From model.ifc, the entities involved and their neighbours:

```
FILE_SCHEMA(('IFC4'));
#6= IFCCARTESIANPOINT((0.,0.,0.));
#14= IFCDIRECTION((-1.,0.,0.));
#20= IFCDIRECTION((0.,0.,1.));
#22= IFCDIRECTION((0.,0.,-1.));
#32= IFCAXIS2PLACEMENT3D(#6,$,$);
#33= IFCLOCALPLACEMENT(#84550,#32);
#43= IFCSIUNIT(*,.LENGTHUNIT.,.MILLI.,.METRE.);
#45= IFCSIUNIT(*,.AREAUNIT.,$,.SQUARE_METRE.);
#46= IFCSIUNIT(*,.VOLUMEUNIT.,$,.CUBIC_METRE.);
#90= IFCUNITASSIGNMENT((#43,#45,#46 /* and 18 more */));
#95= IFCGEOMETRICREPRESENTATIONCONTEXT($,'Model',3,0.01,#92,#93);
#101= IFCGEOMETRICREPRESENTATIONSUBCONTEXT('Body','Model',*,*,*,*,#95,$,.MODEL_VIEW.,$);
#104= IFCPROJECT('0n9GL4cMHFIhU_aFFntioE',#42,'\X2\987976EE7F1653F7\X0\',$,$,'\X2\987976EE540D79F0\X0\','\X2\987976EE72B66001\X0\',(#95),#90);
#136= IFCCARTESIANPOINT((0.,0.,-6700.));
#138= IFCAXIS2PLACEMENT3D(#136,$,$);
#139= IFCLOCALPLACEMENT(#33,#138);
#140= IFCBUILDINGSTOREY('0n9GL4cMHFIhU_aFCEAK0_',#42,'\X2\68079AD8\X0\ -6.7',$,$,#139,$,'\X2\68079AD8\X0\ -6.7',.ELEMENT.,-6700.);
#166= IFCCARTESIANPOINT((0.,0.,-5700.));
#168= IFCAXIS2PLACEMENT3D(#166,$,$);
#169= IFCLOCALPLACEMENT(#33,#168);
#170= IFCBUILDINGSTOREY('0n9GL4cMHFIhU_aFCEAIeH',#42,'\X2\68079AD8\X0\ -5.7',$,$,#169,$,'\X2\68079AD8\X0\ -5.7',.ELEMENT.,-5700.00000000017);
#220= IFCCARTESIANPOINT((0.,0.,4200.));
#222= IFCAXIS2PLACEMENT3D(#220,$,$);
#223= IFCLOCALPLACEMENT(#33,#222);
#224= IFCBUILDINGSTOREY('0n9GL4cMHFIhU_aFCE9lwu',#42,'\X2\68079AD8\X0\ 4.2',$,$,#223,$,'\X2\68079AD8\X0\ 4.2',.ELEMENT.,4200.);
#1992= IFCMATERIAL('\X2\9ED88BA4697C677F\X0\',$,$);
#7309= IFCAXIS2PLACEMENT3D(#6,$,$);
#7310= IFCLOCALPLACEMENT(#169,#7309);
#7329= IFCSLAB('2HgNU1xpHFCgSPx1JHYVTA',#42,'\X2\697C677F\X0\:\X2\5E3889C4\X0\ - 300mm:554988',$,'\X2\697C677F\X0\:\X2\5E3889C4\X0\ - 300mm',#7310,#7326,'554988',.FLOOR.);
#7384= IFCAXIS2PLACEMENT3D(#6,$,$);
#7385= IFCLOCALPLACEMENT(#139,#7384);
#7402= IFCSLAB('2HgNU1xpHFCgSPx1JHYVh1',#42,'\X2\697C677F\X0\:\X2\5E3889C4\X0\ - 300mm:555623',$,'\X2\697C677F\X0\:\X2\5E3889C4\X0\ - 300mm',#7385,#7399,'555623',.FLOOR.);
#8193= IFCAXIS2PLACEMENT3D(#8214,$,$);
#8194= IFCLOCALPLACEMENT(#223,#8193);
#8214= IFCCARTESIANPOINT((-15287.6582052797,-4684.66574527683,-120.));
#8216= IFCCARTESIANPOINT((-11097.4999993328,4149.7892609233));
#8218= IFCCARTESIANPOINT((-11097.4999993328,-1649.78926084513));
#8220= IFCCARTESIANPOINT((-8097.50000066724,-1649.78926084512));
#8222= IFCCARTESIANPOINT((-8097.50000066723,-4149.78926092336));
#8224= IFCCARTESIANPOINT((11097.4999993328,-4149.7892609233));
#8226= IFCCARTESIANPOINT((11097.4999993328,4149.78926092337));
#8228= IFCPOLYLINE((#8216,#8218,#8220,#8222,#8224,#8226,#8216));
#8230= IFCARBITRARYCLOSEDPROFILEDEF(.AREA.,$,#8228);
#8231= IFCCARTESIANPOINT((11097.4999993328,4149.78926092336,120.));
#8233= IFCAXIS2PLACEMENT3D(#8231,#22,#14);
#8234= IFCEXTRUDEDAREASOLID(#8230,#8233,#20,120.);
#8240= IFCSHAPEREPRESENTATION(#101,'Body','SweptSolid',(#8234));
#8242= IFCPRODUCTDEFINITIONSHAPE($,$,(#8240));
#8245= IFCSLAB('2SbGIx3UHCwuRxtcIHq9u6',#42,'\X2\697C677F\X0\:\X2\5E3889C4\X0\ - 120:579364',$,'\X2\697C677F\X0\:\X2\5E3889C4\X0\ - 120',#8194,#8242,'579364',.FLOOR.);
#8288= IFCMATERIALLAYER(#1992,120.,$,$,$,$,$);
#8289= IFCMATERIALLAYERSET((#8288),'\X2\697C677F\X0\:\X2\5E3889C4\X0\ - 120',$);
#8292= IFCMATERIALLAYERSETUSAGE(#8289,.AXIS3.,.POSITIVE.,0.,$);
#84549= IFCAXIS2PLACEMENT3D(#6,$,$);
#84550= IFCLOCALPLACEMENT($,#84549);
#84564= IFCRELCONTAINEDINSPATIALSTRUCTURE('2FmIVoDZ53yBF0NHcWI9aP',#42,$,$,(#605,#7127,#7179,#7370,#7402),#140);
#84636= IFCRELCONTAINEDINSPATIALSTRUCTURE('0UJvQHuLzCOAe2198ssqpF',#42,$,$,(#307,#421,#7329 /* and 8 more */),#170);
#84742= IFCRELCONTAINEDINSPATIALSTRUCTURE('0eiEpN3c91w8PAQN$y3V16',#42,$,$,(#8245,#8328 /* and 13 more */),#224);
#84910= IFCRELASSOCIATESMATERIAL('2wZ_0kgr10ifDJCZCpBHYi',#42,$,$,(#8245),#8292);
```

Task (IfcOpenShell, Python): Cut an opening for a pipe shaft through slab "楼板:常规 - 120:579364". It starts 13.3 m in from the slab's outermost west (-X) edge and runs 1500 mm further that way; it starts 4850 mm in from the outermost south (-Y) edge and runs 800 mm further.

```python
import numpy as np
import ifcopenshell
import ifcopenshell.api.feature
import ifcopenshell.api.geometry
import ifcopenshell.api.root
import ifcopenshell.geom
import ifcopenshell.util.placement
import ifcopenshell.util.representation
import ifcopenshell.util.shape
import ifcopenshell.util.unit

model = ifcopenshell.open("model.ifc")
unit_scale = ifcopenshell.util.unit.calculate_unit_scale(model)
settings = ifcopenshell.geom.settings()


def volume(element):
    """Net volume in cubic metres, openings subtracted."""
    shape = ifcopenshell.geom.create_shape(settings, element)
    return ifcopenshell.util.shape.get_volume(shape.geometry)


slab = model.by_guid("2SbGIx3UHCwuRxtcIHq9u6")
before = volume(slab)

# Extent in the slab's own axes, in metres. The edges named are its -X and -Y sides.
slab_shape = ifcopenshell.geom.create_shape(settings, slab)
vertices = ifcopenshell.util.shape.get_vertices(slab_shape.geometry)
x_min, y_min, bottom = vertices.min(axis=0)
top = vertices[:, 2].max()

opening = ifcopenshell.api.root.create_entity(model, ifc_class="IfcOpeningElement", name="Pipe shaft opening", predefined_type="OPENING")
context = ifcopenshell.util.representation.get_context(model, "Model", "Body", "MODEL_VIEW")
width, depth = 1.5, 0.8
outline = [(0.0, 0.0), (width, 0.0), (width, depth), (0.0, depth), (0.0, 0.0)]
# Overshoot both faces by 50 mm so the cut is clean.
shape = ifcopenshell.api.geometry.add_slab_representation(
    model, context=context, depth=top - bottom + 0.1, polyline=outline
)
ifcopenshell.api.geometry.assign_representation(model, product=opening, representation=shape)

matrix = ifcopenshell.util.placement.get_local_placement(slab.ObjectPlacement)
matrix[:, 3] = matrix @ np.append(np.array([x_min + 13.3, y_min + 4.85, bottom - 0.05]) / unit_scale, 1.0)
ifcopenshell.api.geometry.edit_object_placement(model, product=opening, matrix=matrix, is_si=False)
ifcopenshell.api.feature.add_feature(model, feature=opening, element=slab)

after = volume(slab)

print(f"slab volume {before:.3f} -> {after:.3f} m3")

model.write("model-out.ifc")
```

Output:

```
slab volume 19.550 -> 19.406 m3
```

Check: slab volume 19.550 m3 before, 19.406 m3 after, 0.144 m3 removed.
